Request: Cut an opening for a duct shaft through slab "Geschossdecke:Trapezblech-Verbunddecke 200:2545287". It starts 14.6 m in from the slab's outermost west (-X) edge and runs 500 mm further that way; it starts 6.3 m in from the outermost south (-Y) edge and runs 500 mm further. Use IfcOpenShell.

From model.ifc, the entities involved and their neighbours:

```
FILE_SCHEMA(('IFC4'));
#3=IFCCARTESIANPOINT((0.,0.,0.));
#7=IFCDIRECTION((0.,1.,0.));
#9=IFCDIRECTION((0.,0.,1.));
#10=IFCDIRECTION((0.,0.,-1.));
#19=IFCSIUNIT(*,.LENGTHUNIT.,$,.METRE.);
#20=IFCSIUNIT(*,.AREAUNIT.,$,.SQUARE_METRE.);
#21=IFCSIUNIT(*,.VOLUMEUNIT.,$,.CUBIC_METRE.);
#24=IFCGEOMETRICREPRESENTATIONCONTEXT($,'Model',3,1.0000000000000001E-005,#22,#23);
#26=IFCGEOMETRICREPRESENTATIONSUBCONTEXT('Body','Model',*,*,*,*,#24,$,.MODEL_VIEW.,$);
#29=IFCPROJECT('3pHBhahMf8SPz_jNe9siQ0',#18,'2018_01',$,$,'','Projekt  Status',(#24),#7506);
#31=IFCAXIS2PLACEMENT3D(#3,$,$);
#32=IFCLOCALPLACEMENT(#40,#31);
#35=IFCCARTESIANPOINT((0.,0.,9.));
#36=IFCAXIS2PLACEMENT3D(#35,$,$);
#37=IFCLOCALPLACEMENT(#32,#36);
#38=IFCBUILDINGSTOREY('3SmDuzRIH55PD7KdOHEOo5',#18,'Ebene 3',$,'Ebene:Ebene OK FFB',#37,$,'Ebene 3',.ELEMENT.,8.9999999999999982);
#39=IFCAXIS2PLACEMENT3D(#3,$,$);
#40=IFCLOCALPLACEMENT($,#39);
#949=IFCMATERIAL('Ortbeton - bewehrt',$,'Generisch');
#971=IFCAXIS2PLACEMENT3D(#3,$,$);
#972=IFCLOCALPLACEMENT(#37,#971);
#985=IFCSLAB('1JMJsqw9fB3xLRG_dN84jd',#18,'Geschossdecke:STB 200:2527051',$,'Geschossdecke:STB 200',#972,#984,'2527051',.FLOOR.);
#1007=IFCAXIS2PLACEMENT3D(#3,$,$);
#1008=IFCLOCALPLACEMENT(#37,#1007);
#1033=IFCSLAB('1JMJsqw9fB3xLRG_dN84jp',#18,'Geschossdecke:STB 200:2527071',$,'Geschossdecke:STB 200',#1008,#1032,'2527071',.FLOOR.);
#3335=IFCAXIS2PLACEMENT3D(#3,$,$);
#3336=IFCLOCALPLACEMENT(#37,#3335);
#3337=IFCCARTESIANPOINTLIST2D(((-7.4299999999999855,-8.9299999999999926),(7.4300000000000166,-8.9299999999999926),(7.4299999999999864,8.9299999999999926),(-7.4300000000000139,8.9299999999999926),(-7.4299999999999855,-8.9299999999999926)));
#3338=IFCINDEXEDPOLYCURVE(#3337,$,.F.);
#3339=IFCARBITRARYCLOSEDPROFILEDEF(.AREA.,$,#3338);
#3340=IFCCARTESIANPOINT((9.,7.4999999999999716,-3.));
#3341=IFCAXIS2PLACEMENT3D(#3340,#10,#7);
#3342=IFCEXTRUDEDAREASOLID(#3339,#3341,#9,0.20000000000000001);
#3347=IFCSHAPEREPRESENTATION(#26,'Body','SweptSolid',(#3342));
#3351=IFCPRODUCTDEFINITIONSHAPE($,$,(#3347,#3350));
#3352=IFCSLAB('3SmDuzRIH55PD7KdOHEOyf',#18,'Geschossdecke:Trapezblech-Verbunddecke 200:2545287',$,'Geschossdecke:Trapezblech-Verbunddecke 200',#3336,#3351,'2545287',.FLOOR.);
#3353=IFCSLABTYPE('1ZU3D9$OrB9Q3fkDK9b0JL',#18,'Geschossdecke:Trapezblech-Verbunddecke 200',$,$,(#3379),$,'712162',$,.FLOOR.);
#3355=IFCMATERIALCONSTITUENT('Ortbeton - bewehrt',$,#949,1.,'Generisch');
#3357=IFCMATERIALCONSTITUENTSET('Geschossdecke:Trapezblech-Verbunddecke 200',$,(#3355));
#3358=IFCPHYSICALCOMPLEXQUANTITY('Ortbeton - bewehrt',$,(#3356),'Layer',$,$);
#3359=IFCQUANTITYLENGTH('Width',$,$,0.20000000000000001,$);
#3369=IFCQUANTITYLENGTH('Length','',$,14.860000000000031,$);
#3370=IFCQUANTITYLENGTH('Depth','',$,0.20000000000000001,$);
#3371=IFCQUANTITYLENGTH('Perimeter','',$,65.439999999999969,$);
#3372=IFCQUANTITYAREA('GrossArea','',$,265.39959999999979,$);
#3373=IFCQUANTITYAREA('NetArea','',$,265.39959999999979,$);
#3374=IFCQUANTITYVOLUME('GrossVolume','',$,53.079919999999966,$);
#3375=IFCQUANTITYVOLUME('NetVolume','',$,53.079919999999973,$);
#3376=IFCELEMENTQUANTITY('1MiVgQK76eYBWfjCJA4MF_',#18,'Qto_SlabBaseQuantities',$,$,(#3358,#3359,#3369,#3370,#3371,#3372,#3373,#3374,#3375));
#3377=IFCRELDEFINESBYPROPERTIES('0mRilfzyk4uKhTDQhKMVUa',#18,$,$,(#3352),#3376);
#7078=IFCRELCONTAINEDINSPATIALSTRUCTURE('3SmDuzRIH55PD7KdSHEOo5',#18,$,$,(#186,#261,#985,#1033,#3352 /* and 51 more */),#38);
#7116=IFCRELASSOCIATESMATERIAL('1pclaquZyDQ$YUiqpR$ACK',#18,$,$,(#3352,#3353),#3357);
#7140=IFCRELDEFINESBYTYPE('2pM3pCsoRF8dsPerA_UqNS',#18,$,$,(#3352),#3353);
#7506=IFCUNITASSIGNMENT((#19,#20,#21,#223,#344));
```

```python
import numpy as np
import ifcopenshell
import ifcopenshell.api.feature
import ifcopenshell.api.geometry
import ifcopenshell.api.pset
import ifcopenshell.api.root
import ifcopenshell.geom
import ifcopenshell.util.element
import ifcopenshell.util.placement
import ifcopenshell.util.representation
import ifcopenshell.util.shape
import ifcopenshell.util.unit

model = ifcopenshell.open("model.ifc")
unit_scale = ifcopenshell.util.unit.calculate_unit_scale(model)
area_scale = ifcopenshell.util.unit.calculate_unit_scale(model, "AREAUNIT")
volume_scale = ifcopenshell.util.unit.calculate_unit_scale(model, "VOLUMEUNIT")
settings = ifcopenshell.geom.settings()


def volume(element):
    """Net volume in cubic metres, openings subtracted."""
    shape = ifcopenshell.geom.create_shape(settings, element)
    return ifcopenshell.util.shape.get_volume(shape.geometry)


slab = model.by_guid("3SmDuzRIH55PD7KdOHEOyf")
before = volume(slab)

# Extent in the slab's own axes, in metres. The edges named are its -X and -Y sides.
slab_shape = ifcopenshell.geom.create_shape(settings, slab)
vertices = ifcopenshell.util.shape.get_vertices(slab_shape.geometry)
x_min, y_min, bottom = vertices.min(axis=0)
top = vertices[:, 2].max()

opening = ifcopenshell.api.root.create_entity(model, ifc_class="IfcOpeningElement", name="Duct shaft opening", predefined_type="OPENING")
context = ifcopenshell.util.representation.get_context(model, "Model", "Body", "MODEL_VIEW")
width, depth = 0.5, 0.5
outline = [(0.0, 0.0), (width, 0.0), (width, depth), (0.0, depth), (0.0, 0.0)]
# Overshoot both faces by 50 mm so the cut is clean.
shape = ifcopenshell.api.geometry.add_slab_representation(
    model, context=context, depth=top - bottom + 0.1, polyline=outline
)
ifcopenshell.api.geometry.assign_representation(model, product=opening, representation=shape)

matrix = ifcopenshell.util.placement.get_local_placement(slab.ObjectPlacement)
matrix[:, 3] = matrix @ np.append(np.array([x_min + 14.6, y_min + 6.3, bottom - 0.05]) / unit_scale, 1.0)
ifcopenshell.api.geometry.edit_object_placement(model, product=opening, matrix=matrix, is_si=False)
ifcopenshell.api.feature.add_feature(model, feature=opening, element=slab)

after = volume(slab)

# Update the slab's stored quantities.
qto = model.by_id(ifcopenshell.util.element.get_pset(slab, "Qto_SlabBaseQuantities", should_inherit=False)["id"])
ifcopenshell.api.pset.edit_qto(model, qto=qto, properties={
    "NetArea": after / (top - bottom) / area_scale,
    "NetVolume": after / volume_scale,
})

print(f"slab volume {before:.3f} -> {after:.3f} m3")

model.write("model-out.ifc")
```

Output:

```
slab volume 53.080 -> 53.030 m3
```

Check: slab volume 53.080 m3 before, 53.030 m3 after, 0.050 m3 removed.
